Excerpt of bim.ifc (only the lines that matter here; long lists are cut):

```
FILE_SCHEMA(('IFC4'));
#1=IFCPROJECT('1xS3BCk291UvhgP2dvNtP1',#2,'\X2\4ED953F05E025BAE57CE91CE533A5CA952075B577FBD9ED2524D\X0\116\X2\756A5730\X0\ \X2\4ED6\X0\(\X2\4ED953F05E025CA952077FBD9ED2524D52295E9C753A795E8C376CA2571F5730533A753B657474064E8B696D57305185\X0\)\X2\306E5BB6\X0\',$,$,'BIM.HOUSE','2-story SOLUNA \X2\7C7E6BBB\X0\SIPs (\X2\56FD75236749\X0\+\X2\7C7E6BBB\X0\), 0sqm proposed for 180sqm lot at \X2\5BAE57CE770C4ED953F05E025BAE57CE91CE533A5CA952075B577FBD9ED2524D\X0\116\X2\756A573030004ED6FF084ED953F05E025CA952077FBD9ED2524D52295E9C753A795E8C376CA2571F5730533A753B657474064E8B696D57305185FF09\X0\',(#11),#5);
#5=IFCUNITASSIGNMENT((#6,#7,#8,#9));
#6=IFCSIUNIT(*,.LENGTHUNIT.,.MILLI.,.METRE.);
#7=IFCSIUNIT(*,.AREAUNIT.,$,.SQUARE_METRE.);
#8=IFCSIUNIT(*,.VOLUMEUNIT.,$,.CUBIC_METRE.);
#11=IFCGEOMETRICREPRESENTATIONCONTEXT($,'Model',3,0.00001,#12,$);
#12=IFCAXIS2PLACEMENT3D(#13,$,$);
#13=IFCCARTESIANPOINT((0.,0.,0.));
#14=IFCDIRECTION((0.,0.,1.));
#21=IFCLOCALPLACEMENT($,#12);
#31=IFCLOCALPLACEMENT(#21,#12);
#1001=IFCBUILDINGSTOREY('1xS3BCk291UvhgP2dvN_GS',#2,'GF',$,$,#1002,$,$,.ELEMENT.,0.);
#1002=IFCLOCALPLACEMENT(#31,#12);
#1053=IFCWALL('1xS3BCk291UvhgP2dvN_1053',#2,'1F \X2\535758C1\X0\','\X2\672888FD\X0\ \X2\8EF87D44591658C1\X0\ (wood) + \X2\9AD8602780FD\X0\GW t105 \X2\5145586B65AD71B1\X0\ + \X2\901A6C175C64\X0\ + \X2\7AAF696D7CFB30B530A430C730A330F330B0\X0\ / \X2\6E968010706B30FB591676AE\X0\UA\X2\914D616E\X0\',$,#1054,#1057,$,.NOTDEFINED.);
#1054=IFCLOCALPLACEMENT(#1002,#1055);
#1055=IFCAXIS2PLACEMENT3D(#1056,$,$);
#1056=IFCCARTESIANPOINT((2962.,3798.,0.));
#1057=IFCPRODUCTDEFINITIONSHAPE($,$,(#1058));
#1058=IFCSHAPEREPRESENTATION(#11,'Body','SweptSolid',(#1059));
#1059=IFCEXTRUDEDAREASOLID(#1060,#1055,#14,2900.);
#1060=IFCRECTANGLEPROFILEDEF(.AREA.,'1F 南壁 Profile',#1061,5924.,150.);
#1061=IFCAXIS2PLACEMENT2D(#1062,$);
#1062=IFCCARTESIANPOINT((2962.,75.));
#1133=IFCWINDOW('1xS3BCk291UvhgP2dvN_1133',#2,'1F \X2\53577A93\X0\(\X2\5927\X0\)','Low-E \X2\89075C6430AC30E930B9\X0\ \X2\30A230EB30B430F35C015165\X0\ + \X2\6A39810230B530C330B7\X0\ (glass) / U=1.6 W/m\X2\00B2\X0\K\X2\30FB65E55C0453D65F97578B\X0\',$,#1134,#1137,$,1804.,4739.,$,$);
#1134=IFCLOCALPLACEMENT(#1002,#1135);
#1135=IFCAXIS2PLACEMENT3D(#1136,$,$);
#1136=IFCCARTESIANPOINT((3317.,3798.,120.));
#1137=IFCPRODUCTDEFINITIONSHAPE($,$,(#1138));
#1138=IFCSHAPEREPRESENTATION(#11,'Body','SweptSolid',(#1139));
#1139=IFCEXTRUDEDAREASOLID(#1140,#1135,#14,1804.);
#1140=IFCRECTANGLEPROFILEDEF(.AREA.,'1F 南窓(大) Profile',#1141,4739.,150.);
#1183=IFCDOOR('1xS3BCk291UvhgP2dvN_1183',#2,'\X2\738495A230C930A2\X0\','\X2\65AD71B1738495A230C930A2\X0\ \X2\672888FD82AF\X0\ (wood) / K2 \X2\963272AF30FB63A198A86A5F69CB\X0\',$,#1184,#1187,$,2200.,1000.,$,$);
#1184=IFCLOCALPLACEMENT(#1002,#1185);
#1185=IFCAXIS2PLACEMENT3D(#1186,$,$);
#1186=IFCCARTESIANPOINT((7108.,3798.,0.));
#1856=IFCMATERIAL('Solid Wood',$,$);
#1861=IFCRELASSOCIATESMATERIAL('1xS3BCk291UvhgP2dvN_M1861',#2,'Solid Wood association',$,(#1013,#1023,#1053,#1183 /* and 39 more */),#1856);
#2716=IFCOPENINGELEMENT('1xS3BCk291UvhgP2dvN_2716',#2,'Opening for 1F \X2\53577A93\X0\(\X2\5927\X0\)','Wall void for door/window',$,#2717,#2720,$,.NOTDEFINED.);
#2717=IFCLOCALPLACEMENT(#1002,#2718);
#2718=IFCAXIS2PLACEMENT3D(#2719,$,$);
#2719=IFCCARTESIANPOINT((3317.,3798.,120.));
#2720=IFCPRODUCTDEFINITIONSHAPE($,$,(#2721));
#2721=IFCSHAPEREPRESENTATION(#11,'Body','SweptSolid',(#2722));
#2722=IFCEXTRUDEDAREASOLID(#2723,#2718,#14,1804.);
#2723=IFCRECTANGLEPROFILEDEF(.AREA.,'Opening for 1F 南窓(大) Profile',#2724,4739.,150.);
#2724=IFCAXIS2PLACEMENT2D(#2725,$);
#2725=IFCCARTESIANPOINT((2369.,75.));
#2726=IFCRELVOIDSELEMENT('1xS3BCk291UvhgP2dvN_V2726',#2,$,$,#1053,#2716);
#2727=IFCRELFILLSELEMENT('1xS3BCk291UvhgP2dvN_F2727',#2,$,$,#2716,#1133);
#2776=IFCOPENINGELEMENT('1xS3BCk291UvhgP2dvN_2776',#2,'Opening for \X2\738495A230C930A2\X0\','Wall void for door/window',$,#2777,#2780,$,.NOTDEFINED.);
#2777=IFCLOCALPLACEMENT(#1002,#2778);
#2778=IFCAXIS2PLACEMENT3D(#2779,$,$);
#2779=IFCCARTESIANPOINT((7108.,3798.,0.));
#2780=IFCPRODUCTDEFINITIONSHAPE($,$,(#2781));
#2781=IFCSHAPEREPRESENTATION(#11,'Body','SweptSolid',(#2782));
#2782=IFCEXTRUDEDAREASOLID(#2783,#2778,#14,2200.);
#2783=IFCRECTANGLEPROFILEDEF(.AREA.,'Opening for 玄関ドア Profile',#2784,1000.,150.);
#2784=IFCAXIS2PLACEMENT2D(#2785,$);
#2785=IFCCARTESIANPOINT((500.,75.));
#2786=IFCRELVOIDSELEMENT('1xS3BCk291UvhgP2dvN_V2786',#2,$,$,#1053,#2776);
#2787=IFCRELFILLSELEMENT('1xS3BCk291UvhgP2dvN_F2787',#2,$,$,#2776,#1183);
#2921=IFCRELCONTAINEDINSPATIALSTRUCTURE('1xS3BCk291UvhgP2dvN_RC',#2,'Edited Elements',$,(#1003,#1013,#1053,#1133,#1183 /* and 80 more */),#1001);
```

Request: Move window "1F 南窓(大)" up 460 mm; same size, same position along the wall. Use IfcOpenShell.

```python
import numpy as np
import ifcopenshell
import ifcopenshell.api.geometry
import ifcopenshell.util.placement
import ifcopenshell.util.unit

model = ifcopenshell.open("bim.ifc")
unit_scale = ifcopenshell.util.unit.calculate_unit_scale(model)

window = model.by_guid("1xS3BCk291UvhgP2dvN_1133")
opening = window.FillsVoids[0].RelatingOpeningElement
dz = 460.0

shift = np.array([0.0, 0.0, dz])
# The window is not placed relative to its opening, so move both.
for product in (opening, window):
    matrix = ifcopenshell.util.placement.get_local_placement(product.ObjectPlacement)
    matrix[:3, 3] += shift
    ifcopenshell.api.geometry.edit_object_placement(model, product=product, matrix=matrix, is_si=False)

print(f"moved by {dz * unit_scale:+.3f} m")

model.write("bim_updated.ifc")
```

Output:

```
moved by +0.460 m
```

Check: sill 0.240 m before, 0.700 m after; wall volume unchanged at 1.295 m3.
